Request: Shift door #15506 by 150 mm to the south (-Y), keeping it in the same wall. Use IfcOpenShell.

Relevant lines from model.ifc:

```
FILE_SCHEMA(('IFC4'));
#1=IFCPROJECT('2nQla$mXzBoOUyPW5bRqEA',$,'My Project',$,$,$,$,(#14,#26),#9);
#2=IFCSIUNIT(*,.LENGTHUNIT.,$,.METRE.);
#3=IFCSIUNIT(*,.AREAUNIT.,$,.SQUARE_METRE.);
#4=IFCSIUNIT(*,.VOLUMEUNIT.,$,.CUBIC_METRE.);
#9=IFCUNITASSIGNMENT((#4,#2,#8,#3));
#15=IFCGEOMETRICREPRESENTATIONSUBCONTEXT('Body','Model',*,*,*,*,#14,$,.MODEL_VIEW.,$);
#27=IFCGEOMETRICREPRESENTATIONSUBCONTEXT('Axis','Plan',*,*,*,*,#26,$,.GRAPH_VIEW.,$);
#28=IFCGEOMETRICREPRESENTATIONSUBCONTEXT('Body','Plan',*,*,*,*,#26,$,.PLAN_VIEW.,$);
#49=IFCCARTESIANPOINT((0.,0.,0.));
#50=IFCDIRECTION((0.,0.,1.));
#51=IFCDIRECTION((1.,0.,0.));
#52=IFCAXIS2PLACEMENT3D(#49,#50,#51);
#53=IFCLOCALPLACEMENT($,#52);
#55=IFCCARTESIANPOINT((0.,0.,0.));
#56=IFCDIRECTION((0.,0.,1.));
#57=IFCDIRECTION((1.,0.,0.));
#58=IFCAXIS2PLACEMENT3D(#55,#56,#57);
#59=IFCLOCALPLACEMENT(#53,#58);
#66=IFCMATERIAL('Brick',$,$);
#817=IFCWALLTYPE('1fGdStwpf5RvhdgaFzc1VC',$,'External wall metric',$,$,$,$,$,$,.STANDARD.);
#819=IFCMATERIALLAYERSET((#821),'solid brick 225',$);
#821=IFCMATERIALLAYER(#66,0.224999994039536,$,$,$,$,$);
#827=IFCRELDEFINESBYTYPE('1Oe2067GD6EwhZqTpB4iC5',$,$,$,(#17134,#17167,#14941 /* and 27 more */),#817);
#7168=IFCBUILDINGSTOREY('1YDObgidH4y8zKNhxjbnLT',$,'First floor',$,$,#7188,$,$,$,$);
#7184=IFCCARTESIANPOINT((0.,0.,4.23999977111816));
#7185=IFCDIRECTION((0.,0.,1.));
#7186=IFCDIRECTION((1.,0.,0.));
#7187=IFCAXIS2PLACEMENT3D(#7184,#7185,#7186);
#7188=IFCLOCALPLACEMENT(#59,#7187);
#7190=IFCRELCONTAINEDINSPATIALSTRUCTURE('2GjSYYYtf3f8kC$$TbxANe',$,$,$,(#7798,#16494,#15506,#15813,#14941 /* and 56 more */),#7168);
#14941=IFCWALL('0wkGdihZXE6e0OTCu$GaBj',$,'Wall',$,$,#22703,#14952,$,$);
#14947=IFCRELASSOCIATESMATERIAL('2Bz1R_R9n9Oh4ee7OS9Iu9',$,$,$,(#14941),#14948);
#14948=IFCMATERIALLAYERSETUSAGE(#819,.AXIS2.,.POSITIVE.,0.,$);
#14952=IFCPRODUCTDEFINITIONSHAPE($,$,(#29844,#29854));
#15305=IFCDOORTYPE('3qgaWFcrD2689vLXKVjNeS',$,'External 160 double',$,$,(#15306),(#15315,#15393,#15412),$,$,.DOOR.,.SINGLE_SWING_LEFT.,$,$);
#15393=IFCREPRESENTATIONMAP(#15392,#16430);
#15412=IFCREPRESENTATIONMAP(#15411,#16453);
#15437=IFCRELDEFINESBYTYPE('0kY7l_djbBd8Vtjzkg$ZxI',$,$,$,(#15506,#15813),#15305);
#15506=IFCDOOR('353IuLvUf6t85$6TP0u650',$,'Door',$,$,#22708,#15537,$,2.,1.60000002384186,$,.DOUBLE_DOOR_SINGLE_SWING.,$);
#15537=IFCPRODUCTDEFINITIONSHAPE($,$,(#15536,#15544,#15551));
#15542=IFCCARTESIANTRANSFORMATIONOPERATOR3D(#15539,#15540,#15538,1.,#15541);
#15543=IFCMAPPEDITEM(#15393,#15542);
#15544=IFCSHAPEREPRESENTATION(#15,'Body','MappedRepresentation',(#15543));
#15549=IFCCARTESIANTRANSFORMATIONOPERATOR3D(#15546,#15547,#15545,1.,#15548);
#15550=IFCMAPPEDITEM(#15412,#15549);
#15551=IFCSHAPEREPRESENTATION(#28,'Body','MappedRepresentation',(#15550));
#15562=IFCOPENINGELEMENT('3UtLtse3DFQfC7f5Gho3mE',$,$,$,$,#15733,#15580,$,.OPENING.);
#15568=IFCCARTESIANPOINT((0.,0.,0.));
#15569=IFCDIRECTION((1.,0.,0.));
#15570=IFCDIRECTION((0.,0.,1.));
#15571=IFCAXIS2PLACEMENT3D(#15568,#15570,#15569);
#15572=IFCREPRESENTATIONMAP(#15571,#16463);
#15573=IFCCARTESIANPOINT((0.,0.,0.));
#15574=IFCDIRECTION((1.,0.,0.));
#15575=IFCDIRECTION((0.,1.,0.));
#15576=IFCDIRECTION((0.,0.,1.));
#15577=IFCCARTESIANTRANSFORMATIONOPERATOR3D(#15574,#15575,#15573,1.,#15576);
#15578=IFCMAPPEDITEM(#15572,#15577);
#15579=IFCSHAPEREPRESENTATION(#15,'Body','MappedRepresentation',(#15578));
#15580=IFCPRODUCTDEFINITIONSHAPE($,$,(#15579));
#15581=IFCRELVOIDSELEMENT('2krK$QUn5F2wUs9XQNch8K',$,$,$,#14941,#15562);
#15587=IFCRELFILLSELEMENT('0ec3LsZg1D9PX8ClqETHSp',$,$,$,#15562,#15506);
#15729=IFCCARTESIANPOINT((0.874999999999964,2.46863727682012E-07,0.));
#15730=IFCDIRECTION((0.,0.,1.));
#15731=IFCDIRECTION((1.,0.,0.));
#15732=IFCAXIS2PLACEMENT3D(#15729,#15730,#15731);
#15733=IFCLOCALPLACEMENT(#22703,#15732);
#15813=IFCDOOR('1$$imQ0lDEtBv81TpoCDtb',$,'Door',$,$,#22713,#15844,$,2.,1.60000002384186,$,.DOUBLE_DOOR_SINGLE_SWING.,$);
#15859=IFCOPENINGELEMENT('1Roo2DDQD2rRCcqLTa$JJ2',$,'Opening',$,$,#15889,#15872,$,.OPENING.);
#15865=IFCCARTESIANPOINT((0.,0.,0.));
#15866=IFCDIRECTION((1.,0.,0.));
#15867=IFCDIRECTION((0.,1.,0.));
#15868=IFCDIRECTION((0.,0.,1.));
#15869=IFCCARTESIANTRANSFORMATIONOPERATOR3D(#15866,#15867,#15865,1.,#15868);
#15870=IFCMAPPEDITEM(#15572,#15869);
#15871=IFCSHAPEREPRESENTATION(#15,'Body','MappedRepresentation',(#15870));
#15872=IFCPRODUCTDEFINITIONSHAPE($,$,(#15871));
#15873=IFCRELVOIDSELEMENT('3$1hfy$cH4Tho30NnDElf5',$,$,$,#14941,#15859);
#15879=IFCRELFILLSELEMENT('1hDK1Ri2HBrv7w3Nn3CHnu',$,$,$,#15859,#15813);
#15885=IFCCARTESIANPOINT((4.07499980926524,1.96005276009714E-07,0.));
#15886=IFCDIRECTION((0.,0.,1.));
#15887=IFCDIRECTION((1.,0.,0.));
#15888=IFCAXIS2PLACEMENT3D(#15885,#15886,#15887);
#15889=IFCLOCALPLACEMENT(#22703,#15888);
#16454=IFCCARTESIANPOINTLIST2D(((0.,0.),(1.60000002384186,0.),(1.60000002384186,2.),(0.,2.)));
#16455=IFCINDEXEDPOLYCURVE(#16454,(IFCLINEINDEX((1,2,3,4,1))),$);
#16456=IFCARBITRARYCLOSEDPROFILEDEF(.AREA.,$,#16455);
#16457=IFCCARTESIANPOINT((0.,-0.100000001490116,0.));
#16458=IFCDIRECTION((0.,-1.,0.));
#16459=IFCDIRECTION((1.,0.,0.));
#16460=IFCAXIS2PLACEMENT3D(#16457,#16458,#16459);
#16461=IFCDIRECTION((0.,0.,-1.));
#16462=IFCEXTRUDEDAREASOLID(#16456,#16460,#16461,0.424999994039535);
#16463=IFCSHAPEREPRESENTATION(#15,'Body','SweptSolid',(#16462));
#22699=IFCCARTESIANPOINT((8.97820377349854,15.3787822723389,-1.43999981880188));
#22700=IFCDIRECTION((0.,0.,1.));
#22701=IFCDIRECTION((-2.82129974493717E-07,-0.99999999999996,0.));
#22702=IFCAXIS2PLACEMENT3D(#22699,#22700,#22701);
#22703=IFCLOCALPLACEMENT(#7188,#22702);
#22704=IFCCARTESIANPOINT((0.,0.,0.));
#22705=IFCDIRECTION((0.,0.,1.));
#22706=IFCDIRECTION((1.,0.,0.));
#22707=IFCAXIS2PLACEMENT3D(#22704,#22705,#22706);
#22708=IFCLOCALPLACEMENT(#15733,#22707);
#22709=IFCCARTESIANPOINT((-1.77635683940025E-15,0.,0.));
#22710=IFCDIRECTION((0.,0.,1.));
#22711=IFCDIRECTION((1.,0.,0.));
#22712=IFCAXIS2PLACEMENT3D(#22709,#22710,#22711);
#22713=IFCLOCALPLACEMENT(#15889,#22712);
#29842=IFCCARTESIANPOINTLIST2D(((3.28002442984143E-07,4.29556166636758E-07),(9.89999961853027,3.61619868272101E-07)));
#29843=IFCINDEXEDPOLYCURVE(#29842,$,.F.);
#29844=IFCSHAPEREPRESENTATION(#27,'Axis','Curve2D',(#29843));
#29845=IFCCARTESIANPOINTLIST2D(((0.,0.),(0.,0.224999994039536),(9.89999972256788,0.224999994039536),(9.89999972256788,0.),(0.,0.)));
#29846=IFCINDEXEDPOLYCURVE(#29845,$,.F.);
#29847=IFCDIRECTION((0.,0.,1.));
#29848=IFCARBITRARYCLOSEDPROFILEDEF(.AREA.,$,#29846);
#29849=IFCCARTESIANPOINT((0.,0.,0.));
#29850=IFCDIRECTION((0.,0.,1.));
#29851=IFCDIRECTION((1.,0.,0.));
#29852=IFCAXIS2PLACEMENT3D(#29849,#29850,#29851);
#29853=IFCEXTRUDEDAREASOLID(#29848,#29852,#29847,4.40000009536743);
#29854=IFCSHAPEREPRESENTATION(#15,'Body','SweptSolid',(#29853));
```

```python
import ifcopenshell
import ifcopenshell.api.geometry
import ifcopenshell.util.placement
import ifcopenshell.util.unit

model = ifcopenshell.open("model.ifc")
unit_scale = ifcopenshell.util.unit.calculate_unit_scale(model)

door = model.by_guid("353IuLvUf6t85$6TP0u650")
opening = door.FillsVoids[0].RelatingOpeningElement
wall = opening.VoidsElements[0].RelatingBuildingElement

wall_matrix = ifcopenshell.util.placement.get_local_placement(wall.ObjectPlacement)
shift = wall_matrix[:3, 0] * 0.15 / unit_scale
before = ifcopenshell.util.placement.get_local_placement(door.ObjectPlacement)[:3, 3].copy()

# The door is placed relative to its opening, so it follows when the opening moves.
matrix = ifcopenshell.util.placement.get_local_placement(opening.ObjectPlacement)
matrix[:3, 3] += shift
ifcopenshell.api.geometry.edit_object_placement(
    model, product=opening, matrix=matrix, is_si=False, should_transform_children=True
)

after = ifcopenshell.util.placement.get_local_placement(door.ObjectPlacement)[:3, 3]
print("door moved by", (after - before).round(3) + 0.0)

model.write("model-out.ifc")
```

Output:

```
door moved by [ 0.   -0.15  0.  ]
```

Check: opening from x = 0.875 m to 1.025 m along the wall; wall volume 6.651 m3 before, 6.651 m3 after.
